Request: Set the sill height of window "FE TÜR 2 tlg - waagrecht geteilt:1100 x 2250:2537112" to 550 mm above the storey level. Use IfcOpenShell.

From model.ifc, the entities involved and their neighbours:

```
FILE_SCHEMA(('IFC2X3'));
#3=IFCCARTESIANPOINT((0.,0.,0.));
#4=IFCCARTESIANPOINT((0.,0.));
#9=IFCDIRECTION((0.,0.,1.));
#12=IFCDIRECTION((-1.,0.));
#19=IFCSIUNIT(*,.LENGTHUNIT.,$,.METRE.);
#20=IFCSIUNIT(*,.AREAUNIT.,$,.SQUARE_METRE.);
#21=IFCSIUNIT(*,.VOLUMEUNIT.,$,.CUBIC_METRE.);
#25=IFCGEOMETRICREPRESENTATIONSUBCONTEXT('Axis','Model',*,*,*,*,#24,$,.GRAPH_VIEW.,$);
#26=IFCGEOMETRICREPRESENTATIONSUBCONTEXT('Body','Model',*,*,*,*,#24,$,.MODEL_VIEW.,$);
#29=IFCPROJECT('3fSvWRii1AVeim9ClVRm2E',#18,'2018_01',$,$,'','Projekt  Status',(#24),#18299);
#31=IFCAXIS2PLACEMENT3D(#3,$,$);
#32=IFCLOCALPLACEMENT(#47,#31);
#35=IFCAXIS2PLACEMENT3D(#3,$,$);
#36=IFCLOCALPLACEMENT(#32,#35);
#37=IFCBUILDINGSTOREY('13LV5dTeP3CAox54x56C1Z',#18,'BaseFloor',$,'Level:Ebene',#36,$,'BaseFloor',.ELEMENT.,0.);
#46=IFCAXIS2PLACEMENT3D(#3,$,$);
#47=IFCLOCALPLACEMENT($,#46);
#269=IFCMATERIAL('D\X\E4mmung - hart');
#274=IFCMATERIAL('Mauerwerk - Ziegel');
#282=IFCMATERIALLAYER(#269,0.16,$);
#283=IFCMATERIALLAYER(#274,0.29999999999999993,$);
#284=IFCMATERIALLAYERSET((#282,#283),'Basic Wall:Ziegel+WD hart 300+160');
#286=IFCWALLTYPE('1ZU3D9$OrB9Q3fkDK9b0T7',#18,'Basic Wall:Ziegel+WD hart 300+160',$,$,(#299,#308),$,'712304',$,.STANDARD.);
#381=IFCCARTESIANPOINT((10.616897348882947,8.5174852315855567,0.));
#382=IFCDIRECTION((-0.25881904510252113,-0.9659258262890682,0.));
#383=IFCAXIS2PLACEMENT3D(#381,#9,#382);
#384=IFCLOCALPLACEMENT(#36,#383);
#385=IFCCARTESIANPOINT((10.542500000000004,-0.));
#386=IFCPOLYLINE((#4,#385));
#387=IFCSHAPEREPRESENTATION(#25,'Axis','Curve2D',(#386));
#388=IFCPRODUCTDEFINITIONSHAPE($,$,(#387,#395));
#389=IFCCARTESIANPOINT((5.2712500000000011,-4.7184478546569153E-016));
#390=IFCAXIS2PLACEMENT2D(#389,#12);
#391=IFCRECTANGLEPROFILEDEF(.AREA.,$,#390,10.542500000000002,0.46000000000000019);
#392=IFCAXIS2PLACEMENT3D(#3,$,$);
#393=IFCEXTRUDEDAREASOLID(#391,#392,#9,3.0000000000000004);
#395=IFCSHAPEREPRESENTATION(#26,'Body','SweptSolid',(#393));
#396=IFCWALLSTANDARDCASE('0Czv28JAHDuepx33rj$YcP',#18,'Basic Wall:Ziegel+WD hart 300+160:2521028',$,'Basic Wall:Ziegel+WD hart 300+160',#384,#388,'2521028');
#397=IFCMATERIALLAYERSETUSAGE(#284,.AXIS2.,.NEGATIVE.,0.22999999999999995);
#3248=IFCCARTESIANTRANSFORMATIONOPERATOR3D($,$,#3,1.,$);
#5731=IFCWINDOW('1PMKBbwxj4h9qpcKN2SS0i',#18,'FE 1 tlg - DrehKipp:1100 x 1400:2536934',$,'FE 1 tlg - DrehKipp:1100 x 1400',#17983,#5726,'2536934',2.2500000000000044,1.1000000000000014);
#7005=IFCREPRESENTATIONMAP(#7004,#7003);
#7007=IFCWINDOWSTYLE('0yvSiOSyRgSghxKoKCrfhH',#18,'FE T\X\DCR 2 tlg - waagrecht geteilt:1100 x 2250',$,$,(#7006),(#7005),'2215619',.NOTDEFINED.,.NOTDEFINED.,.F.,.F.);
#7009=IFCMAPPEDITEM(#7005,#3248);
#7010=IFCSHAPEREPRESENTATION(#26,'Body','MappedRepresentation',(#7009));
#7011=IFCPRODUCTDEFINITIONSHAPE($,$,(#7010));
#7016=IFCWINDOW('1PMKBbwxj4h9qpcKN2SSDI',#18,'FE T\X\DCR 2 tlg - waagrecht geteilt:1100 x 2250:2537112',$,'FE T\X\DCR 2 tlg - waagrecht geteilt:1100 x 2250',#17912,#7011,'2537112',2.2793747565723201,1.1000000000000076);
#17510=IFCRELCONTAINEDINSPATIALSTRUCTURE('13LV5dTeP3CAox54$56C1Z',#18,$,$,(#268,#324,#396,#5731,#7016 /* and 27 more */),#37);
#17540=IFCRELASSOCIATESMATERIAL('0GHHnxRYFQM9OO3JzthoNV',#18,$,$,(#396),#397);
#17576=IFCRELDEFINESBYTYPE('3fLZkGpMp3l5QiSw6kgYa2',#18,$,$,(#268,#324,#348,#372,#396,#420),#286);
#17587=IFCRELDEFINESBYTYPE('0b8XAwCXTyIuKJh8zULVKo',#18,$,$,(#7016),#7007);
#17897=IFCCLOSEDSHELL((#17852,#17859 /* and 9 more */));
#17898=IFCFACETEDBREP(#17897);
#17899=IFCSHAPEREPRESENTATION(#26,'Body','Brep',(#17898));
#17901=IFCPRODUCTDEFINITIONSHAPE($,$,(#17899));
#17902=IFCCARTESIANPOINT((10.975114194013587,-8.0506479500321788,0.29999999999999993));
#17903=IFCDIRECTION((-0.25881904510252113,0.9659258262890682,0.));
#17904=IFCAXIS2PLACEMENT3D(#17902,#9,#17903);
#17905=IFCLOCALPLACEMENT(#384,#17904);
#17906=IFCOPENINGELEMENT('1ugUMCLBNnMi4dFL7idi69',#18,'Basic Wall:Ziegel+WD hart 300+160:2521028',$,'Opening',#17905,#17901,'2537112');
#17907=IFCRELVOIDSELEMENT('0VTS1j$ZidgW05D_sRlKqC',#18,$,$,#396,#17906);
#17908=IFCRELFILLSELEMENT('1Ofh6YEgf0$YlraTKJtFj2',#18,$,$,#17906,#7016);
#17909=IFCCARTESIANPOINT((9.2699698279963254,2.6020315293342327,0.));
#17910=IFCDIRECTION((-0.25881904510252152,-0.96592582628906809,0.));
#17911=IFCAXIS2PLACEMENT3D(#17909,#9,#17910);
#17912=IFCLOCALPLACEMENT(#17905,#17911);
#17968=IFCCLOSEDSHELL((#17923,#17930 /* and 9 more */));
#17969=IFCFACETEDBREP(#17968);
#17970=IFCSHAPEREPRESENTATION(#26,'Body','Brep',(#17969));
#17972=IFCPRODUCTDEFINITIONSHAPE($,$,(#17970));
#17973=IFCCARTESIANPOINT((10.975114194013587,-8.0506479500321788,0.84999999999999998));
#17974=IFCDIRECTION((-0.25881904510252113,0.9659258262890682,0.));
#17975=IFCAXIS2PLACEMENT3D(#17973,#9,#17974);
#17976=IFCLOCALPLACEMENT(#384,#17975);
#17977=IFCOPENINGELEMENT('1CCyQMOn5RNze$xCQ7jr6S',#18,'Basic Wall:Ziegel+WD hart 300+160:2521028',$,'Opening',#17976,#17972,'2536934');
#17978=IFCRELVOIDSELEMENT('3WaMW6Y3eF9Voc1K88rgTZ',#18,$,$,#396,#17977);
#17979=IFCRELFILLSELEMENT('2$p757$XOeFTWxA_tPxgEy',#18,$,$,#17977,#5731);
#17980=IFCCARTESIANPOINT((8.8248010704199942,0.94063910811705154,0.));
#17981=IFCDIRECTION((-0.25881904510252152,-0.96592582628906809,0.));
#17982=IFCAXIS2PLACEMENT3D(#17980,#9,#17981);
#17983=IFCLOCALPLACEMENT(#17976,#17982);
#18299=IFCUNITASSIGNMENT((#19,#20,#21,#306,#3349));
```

```python
import numpy as np
import ifcopenshell
import ifcopenshell.api.geometry
import ifcopenshell.geom
import ifcopenshell.util.element
import ifcopenshell.util.placement
import ifcopenshell.util.shape
import ifcopenshell.util.unit

model = ifcopenshell.open("model.ifc")
unit_scale = ifcopenshell.util.unit.calculate_unit_scale(model)

window = model.by_id(7016)
opening = window.FillsVoids[0].RelatingOpeningElement
storey = ifcopenshell.util.element.get_container(window, ifc_class="IfcBuildingStorey")
level = ifcopenshell.util.placement.get_local_placement(storey.ObjectPlacement)[2, 3]

# The opening's origin need not be at the sill, so measure its lowest point.
shape = ifcopenshell.geom.create_shape(ifcopenshell.geom.settings(), opening)
bottom = ifcopenshell.util.shape.get_shape_bottom_elevation(shape, shape.geometry) / unit_scale
dz = level + 0.55 / unit_scale - bottom

shift = np.array([0.0, 0.0, dz])
# The window is placed relative to its opening, so it follows when the opening moves.
matrix = ifcopenshell.util.placement.get_local_placement(opening.ObjectPlacement)
matrix[:3, 3] += shift
ifcopenshell.api.geometry.edit_object_placement(
    model, product=opening, matrix=matrix, is_si=False, should_transform_children=True
)

print(f"moved by {dz * unit_scale:+.3f} m")

model.write("model_edited.ifc")
```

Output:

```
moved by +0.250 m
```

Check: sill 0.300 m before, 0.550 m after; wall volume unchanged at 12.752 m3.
